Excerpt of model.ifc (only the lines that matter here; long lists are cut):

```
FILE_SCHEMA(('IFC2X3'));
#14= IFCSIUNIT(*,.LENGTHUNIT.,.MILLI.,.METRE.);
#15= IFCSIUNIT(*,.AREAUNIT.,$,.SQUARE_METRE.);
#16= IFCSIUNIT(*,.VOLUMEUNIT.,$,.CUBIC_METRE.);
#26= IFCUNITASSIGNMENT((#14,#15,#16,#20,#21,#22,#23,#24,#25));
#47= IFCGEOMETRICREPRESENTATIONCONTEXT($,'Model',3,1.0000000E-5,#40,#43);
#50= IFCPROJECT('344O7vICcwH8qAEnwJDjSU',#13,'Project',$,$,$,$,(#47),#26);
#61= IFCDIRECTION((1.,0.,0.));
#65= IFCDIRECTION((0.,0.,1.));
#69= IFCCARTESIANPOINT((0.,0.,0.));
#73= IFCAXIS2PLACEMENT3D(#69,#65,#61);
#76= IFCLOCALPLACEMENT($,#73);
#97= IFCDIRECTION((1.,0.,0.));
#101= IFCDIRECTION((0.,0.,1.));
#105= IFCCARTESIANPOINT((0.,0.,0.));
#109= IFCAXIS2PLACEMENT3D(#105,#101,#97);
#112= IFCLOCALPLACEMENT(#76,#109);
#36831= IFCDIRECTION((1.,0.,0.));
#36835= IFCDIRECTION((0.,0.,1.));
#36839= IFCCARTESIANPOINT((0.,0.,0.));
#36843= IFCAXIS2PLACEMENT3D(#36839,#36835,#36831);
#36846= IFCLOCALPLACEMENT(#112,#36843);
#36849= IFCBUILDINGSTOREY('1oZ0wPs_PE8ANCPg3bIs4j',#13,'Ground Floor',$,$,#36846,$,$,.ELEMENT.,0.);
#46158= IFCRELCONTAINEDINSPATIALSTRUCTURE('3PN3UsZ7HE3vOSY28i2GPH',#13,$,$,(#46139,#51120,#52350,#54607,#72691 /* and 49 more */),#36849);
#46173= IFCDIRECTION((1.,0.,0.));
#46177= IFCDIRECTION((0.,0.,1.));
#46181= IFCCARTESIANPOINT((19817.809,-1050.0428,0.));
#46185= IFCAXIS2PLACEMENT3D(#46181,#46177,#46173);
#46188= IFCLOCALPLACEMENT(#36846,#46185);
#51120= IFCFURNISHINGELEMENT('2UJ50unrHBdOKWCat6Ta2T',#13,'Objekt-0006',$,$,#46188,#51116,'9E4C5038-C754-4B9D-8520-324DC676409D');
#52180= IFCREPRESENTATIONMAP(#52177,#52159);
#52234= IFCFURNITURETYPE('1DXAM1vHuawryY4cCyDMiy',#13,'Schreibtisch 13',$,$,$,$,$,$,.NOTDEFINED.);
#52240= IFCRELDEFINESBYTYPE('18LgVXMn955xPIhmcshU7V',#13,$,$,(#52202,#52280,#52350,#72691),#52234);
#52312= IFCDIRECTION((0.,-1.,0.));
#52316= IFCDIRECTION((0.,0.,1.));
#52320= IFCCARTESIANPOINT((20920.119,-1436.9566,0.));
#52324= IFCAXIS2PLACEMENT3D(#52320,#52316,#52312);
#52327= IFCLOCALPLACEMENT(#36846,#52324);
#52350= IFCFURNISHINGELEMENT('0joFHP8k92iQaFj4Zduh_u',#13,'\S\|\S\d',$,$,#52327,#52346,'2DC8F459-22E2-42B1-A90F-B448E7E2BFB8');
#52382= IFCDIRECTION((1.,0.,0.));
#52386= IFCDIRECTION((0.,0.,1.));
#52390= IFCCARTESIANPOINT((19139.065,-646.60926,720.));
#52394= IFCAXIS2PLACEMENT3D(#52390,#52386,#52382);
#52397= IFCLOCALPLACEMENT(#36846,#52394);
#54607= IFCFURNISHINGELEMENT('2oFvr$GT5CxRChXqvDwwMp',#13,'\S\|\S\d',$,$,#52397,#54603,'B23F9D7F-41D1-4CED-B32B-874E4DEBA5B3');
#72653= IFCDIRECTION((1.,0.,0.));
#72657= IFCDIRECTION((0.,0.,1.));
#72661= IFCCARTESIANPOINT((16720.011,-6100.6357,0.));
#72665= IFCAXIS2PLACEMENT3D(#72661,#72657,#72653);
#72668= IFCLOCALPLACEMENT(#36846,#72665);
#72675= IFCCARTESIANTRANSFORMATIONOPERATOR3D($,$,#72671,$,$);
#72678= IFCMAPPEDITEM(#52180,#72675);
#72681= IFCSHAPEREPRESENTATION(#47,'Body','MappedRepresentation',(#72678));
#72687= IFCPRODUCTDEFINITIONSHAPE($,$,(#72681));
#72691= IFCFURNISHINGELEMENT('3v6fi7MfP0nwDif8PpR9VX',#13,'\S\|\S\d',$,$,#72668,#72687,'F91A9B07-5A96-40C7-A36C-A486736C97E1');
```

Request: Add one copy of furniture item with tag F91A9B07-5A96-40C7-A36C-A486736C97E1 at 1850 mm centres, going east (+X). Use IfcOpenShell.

```python
import numpy as np
import ifcopenshell
import ifcopenshell.api.geometry
import ifcopenshell.api.root
import ifcopenshell.util.element
import ifcopenshell.util.placement
import ifcopenshell.util.unit

model = ifcopenshell.open("model.ifc")
unit_scale = ifcopenshell.util.unit.calculate_unit_scale(model)


def reuse_history(source, copy):
    """copy_class also copies each property set's owner history, people and application; keep the originals."""
    for rel in copy.IsDefinedBy:
        if rel.is_a("IfcRelDefinesByProperties") and (history := rel.RelatingPropertyDefinition.OwnerHistory):
            rel.RelatingPropertyDefinition.OwnerHistory = source.OwnerHistory
            ifcopenshell.util.element.remove_deep2(model, history)


source = model.by_guid("3v6fi7MfP0nwDif8PpR9VX")
base = ifcopenshell.util.placement.get_local_placement(source.ObjectPlacement)
step = np.array([1.0, 0.0, 0.0]) * 1.85 / unit_scale

for i in range(1, 2):
    copy = ifcopenshell.api.root.copy_class(model, product=source)
    copy.Representation = ifcopenshell.util.element.copy_deep(
        model, source.Representation, exclude=["IfcGeometricRepresentationContext", "IfcRepresentationMap"]
    )
    copy.Tag = None
    reuse_history(source, copy)
    matrix = base.copy()
    matrix[:3, 3] += i * step
    print("added at", matrix[:3, 3].round(3) + 0.0)
    ifcopenshell.api.geometry.edit_object_placement(model, product=copy, matrix=matrix, is_si=False)

model.write("model_updated.ifc")
```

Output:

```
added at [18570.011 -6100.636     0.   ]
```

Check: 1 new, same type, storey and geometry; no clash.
